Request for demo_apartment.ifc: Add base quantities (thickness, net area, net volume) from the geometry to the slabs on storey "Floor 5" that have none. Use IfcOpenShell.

First a look at what the model holds.

```python
import ifcopenshell
import ifcopenshell.util.element
import ifcopenshell.util.unit

model = ifcopenshell.open("demo_apartment.ifc")
print(model.schema)
for unit_type in ("LENGTHUNIT", "AREAUNIT", "VOLUMEUNIT"):
    print(unit_type, ifcopenshell.util.unit.calculate_unit_scale(model, unit_type))
storey = next(s for s in model.by_type("IfcBuildingStorey") if s.Name == "Floor 5")
slabs = [e for e in ifcopenshell.util.element.get_decomposition(storey) if e.is_a("IfcSlab")]
for e in sorted(slabs, key=lambda e: e.id()):
    print(e.id(), e.is_a(), e.Name, list(ifcopenshell.util.element.get_psets(e, qtos_only=True)), sep=" | ")
```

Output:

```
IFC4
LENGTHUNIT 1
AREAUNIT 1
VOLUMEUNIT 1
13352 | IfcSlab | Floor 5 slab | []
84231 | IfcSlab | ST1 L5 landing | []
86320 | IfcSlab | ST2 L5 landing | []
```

```python
import ifcopenshell
import ifcopenshell.api.pset
import ifcopenshell.geom
import ifcopenshell.util.element
import ifcopenshell.util.shape
import ifcopenshell.util.unit

model = ifcopenshell.open("demo_apartment.ifc")
unit_scale = ifcopenshell.util.unit.calculate_unit_scale(model)
area_scale = ifcopenshell.util.unit.calculate_unit_scale(model, "AREAUNIT")
volume_scale = ifcopenshell.util.unit.calculate_unit_scale(model, "VOLUMEUNIT")
settings = ifcopenshell.geom.settings()

storey = next(s for s in model.by_type("IfcBuildingStorey") if s.Name == "Floor 5")
slabs = [e for e in ifcopenshell.util.element.get_decomposition(storey) if e.is_a("IfcSlab")]

for e in sorted(slabs, key=lambda e: e.id()):
    if ifcopenshell.util.element.get_psets(e, qtos_only=True, should_inherit=False):
        continue
    # Geometry comes back in metres, in the element's own axes.
    shape = ifcopenshell.geom.create_shape(settings, e)
    values = {
        "Width": ifcopenshell.util.shape.get_z(shape.geometry) / unit_scale,
        "NetArea": ifcopenshell.util.shape.get_footprint_area(shape.geometry) / area_scale,
        "NetVolume": ifcopenshell.util.shape.get_volume(shape.geometry) / volume_scale,
    }
    qto = ifcopenshell.api.pset.add_qto(model, product=e, name="Qto_SlabBaseQuantities")
    ifcopenshell.api.pset.edit_qto(model, qto=qto, properties=values)
    print(e.id(), {k: round(v, 3) for k, v in values.items()})

model.write("demo_apartment_v2.ifc")
```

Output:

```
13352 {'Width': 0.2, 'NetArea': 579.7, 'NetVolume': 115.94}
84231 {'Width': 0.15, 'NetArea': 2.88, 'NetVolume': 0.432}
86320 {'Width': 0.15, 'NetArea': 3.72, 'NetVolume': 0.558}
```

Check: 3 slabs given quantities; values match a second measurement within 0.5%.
